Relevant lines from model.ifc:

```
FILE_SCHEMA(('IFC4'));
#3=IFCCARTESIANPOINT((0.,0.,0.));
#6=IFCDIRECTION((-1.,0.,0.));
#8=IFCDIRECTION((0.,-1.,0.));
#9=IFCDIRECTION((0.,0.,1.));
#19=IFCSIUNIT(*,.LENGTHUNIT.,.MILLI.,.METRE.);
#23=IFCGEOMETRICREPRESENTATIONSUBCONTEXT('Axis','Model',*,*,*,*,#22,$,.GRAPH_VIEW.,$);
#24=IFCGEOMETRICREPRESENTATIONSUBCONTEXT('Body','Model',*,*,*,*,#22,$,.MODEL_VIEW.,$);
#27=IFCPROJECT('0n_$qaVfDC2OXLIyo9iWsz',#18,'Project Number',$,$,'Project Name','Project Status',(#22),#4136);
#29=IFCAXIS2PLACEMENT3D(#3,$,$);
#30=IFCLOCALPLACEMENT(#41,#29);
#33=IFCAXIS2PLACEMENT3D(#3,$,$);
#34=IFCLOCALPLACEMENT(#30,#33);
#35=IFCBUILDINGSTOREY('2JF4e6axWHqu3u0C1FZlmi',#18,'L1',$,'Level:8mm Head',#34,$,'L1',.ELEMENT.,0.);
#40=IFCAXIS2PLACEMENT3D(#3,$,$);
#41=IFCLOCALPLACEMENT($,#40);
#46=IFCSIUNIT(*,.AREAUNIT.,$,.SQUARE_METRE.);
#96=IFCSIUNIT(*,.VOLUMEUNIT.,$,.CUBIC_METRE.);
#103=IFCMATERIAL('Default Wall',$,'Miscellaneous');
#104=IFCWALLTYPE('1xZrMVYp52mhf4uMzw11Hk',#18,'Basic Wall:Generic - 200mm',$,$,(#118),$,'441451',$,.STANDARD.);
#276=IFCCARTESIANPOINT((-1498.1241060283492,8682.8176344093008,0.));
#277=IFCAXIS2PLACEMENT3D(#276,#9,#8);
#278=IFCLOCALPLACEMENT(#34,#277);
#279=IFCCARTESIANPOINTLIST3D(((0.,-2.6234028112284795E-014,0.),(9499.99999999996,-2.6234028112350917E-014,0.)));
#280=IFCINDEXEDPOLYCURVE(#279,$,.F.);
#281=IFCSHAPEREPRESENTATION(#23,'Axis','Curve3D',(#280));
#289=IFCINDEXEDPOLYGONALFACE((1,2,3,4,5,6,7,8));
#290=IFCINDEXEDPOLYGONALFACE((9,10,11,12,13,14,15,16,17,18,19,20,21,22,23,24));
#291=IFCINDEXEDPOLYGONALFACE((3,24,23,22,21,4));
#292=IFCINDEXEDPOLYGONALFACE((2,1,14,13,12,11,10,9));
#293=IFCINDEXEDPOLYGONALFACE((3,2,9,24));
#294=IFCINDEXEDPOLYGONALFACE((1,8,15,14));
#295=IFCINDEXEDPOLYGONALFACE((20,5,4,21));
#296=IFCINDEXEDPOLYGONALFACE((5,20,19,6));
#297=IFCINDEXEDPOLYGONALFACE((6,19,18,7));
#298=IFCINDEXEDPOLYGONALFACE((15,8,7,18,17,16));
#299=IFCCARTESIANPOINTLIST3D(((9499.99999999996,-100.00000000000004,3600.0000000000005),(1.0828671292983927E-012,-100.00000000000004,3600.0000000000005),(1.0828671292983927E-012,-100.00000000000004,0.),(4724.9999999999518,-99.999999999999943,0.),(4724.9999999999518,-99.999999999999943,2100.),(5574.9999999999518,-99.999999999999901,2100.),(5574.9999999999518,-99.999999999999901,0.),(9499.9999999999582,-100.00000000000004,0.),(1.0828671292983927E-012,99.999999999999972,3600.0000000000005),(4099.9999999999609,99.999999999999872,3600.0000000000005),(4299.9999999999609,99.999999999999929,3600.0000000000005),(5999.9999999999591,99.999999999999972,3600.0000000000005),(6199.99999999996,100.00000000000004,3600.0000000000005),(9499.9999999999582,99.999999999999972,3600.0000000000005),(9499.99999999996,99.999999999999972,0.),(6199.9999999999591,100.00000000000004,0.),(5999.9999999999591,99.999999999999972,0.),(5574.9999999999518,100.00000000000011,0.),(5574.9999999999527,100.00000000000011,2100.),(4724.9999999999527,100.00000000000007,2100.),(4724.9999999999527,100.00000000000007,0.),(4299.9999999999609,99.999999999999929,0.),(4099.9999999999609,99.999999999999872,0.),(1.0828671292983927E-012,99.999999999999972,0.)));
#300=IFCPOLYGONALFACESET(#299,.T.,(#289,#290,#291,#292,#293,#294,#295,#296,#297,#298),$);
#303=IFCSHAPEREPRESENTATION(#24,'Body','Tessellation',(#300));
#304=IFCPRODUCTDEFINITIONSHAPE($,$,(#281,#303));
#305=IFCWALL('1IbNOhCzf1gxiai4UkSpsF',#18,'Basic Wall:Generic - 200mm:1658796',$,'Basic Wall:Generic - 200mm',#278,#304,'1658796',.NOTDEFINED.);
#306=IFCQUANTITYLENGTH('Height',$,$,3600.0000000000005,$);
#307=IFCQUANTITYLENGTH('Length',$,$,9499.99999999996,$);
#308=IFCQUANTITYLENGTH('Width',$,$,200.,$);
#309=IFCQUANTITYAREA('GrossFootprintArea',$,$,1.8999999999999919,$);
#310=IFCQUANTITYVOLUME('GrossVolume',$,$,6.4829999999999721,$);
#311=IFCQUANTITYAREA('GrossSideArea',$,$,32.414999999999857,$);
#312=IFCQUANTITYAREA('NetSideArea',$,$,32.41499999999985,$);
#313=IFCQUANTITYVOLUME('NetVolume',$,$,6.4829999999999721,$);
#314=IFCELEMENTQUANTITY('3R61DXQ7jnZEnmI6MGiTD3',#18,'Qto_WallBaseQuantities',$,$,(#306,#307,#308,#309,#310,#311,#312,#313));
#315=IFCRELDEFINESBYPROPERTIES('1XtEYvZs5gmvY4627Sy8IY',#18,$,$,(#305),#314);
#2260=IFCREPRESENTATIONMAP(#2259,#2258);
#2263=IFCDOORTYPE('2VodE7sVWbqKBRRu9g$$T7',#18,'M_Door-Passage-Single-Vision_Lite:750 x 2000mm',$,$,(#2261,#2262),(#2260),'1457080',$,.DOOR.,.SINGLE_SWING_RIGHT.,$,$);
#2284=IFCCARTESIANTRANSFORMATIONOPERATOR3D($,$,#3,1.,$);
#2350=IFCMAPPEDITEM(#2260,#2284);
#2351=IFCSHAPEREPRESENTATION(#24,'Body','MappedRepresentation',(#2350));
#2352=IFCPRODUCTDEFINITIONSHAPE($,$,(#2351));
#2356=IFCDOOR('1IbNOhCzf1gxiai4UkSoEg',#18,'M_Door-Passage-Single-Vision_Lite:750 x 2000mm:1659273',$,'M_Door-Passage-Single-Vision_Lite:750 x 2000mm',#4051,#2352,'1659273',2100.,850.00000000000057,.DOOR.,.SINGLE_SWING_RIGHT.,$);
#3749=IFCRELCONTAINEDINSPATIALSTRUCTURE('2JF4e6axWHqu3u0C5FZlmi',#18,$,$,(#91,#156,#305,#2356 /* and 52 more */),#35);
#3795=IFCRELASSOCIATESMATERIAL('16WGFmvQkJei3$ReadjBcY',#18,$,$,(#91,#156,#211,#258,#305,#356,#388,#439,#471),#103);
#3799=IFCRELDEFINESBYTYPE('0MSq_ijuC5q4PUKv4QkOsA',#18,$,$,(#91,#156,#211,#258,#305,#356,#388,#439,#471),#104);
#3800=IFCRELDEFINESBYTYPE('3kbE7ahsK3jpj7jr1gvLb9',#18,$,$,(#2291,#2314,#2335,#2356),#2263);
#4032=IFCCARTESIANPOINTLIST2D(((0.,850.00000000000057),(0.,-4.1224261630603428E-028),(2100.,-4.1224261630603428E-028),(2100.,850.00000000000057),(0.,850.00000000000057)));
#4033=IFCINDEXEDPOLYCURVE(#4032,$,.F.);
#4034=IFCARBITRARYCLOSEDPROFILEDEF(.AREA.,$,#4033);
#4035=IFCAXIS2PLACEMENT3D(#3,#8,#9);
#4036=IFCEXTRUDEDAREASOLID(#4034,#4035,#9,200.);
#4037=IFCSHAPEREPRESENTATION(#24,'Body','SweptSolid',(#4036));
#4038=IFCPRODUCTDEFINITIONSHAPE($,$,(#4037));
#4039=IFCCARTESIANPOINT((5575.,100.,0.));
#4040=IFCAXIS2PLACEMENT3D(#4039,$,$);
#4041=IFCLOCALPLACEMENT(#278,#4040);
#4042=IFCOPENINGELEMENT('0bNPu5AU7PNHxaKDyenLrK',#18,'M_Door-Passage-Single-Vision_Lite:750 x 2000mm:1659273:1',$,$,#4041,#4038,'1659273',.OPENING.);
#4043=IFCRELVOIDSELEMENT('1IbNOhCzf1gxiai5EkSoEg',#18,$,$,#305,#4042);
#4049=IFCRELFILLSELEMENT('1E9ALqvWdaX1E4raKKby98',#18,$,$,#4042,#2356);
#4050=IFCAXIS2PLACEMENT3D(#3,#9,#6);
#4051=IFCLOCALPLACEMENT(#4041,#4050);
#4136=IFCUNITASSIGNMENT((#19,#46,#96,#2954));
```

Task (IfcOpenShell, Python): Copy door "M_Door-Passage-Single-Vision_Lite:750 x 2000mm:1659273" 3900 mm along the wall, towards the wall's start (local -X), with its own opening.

```python
import ifcopenshell
import ifcopenshell.api.feature
import ifcopenshell.api.geometry
import ifcopenshell.api.pset
import ifcopenshell.api.root
import ifcopenshell.geom
import ifcopenshell.util.element
import ifcopenshell.util.placement
import ifcopenshell.util.shape
import ifcopenshell.util.unit

model = ifcopenshell.open("model.ifc")
unit_scale = ifcopenshell.util.unit.calculate_unit_scale(model)
area_scale = ifcopenshell.util.unit.calculate_unit_scale(model, "AREAUNIT")
volume_scale = ifcopenshell.util.unit.calculate_unit_scale(model, "VOLUMEUNIT")
settings = ifcopenshell.geom.settings()


def volume(element):
    """Net volume in cubic metres, openings subtracted."""
    shape = ifcopenshell.geom.create_shape(settings, element)
    return ifcopenshell.util.shape.get_volume(shape.geometry)


def reuse_history(source, copy):
    """copy_class also copies each property set's owner history, people and application; keep the originals."""
    for rel in copy.IsDefinedBy:
        if rel.is_a("IfcRelDefinesByProperties") and (history := rel.RelatingPropertyDefinition.OwnerHistory):
            rel.RelatingPropertyDefinition.OwnerHistory = source.OwnerHistory
            ifcopenshell.util.element.remove_deep2(model, history)


door = model.by_guid("1IbNOhCzf1gxiai4UkSoEg")
opening = door.FillsVoids[0].RelatingOpeningElement
wall = opening.VoidsElements[0].RelatingBuildingElement
before = volume(wall)
shift = ifcopenshell.util.placement.get_local_placement(wall.ObjectPlacement)[:3, 0] * -3.9 / unit_scale

# copy_class copies the void relationship, type, container and properties, but no geometry.
new_opening = ifcopenshell.api.root.copy_class(model, product=opening)
new_opening.Representation = ifcopenshell.util.element.copy_deep(
    model, opening.Representation, exclude=["IfcGeometricRepresentationContext", "IfcRepresentationMap"]
)
new_opening.Name = "M_Door-Passage-Single-Vision_Lite:750 x 2000mm"
new_opening.Tag = None
reuse_history(opening, new_opening)
new_door = ifcopenshell.api.root.copy_class(model, product=door)
new_door.Representation = ifcopenshell.util.element.copy_deep(
    model, door.Representation, exclude=["IfcGeometricRepresentationContext", "IfcRepresentationMap"]
)
new_door.Name = "M_Door-Passage-Single-Vision_Lite:750 x 2000mm"
new_door.Tag = None
reuse_history(door, new_door)
ifcopenshell.api.feature.add_filling(model, opening=new_opening, element=new_door)

for old, new in ((opening, new_opening), (door, new_door)):
    matrix = ifcopenshell.util.placement.get_local_placement(old.ObjectPlacement)
    matrix[:3, 3] += shift
    ifcopenshell.api.geometry.edit_object_placement(model, product=new, matrix=matrix, is_si=False)

after = volume(wall)
thickness = 0.2  # wall thickness in metres

# Update the wall's stored quantities.
qto = model.by_id(ifcopenshell.util.element.get_pset(wall, "Qto_WallBaseQuantities", should_inherit=False)["id"])
ifcopenshell.api.pset.edit_qto(model, qto=qto, properties={
    "NetSideArea": after / thickness / area_scale,
    "NetVolume": after / volume_scale,
})

print(f"wall volume {before:.3f} -> {after:.3f} m3")

model.write("model_updated.ifc")
```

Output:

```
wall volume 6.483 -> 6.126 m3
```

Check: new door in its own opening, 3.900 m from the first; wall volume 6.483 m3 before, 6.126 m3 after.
